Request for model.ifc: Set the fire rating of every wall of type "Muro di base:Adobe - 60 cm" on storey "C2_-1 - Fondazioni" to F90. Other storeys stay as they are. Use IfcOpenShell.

First a look at what the model holds.

```python
import ifcopenshell
import ifcopenshell.util.element

model = ifcopenshell.open("model.ifc")
print(model.schema)
storey = next(s for s in model.by_type("IfcBuildingStorey") if s.Name == "C2_-1 - Fondazioni")
walls = [e for e in ifcopenshell.util.element.get_decomposition(storey) if e.is_a("IfcWall")]
seen = {}
for e in walls:
    element_type = ifcopenshell.util.element.get_type(e)
    key = (element_type.Name if element_type != e and element_type else None, ifcopenshell.util.element.get_pset(e, "Pset_WallCommon", "FireRating"))
    seen[key] = seen.get(key, 0) + 1
for (name, value), count in sorted(seen.items(), key=str):
    print(count, "x", name, "|", value)
```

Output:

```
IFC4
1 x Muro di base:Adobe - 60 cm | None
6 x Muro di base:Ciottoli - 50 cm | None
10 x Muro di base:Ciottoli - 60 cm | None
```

```python
import ifcopenshell
import ifcopenshell.api.pset
import ifcopenshell.util.element

model = ifcopenshell.open("model.ifc")

storey = next(s for s in model.by_type("IfcBuildingStorey") if s.Name == "C2_-1 - Fondazioni")
walls = [e for e in ifcopenshell.util.element.get_decomposition(storey) if e.is_a("IfcWall")]

count = 0
for e in walls:
    element_type = ifcopenshell.util.element.get_type(e)
    if element_type in (None, e) or element_type.Name != "Muro di base:Adobe - 60 cm":
        continue
    # add_pset returns the element's existing set when there is one.
    pset = ifcopenshell.api.pset.add_pset(model, product=e, name="Pset_WallCommon")
    ifcopenshell.api.pset.edit_pset(model, pset=pset, properties={"FireRating": "F90"})
    count += 1

print(count, "walls updated")

model.write("model_edited.ifc")
```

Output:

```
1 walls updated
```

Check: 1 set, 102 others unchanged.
